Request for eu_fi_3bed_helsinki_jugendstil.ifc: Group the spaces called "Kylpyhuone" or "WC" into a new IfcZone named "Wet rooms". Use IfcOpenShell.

First a look at what the model holds.

```python
import ifcopenshell

model = ifcopenshell.open("eu_fi_3bed_helsinki_jugendstil.ifc")
print(model.schema)
seen = {}
for space in model.by_type("IfcSpace"):
    seen[space.LongName] = seen.get(space.LongName, 0) + 1
for name, count in sorted(seen.items(), key=str):
    print(count, "x", name)
print("zones:", [z.Name for z in model.by_type("IfcZone")][:20])
```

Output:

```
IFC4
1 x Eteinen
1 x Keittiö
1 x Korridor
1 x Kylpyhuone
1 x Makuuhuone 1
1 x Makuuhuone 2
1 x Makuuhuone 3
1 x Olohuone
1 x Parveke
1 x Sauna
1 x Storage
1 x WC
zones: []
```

```python
import ifcopenshell
import ifcopenshell.api.group
import ifcopenshell.api.root

model = ifcopenshell.open("eu_fi_3bed_helsinki_jugendstil.ifc")

names = {"Kylpyhuone", "WC"}
spaces = [s for s in model.by_type("IfcSpace") if s.LongName in names]

zone = ifcopenshell.api.root.create_entity(model, ifc_class="IfcZone", name="Wet rooms")
ifcopenshell.api.group.assign_group(model, products=spaces, group=zone)
print(len(spaces), "spaces in", zone.Name)

model.write("eu_fi_3bed_helsinki_jugendstil_edited.ifc")
```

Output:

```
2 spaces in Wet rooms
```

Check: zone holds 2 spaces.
